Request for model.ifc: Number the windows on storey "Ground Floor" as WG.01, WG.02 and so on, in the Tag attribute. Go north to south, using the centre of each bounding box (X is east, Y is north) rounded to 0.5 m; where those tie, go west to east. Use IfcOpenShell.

First a look at what the model holds.

```python
import ifcopenshell
import ifcopenshell.util.element
import ifcopenshell.util.placement

model = ifcopenshell.open("model.ifc")
print(model.schema)
storey = next(s for s in model.by_type("IfcBuildingStorey") if s.Name == "Ground Floor")
windows = [e for e in ifcopenshell.util.element.get_decomposition(storey) if e.is_a("IfcWindow")]
for e in sorted(windows, key=lambda e: e.id()):
    origin = ifcopenshell.util.placement.get_local_placement(e.ObjectPlacement)[:3, 3]
    print(e.id(), e.Tag, e.Name, origin.round(2) + 0.0, sep=" | ")
```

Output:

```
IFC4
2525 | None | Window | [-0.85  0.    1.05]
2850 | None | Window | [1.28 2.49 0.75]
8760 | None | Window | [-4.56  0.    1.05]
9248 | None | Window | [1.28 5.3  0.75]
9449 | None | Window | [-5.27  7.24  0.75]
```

```python
import ifcopenshell
import ifcopenshell.geom
import ifcopenshell.util.element
import ifcopenshell.util.shape

model = ifcopenshell.open("model.ifc")
settings = ifcopenshell.geom.settings()
settings.set("use-world-coords", True)


def centre(element):
    shape = ifcopenshell.geom.create_shape(settings, element)
    return ifcopenshell.util.shape.get_bbox_centroid(shape.geometry)


storey = next(s for s in model.by_type("IfcBuildingStorey") if s.Name == "Ground Floor")
windows = [e for e in ifcopenshell.util.element.get_decomposition(storey) if e.is_a("IfcWindow")]

# Insertion points can sit at a corner or the storey origin, so sort by the geometry (in metres).
centres = {e: centre(e) for e in windows}
windows.sort(key=lambda e: (-round(centres[e][1] / 0.5), centres[e][0]))

for i, e in enumerate(windows, start=1):
    number = f"WG.{i:02d}"
    e.Tag = number
    print(e.id(), number)

model.write("model-out.ifc")
```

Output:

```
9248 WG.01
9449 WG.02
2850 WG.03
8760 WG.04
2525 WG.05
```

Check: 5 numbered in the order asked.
